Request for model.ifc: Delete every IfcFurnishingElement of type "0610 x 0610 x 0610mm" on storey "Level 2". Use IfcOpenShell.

First a look at what the model holds.

```python
import ifcopenshell
import ifcopenshell.util.element

model = ifcopenshell.open("model.ifc")
print(model.schema)
storey = next(s for s in model.by_type("IfcBuildingStorey") if s.Name == "Level 2")
furniture = [e for e in ifcopenshell.util.element.get_decomposition(storey) if e.is_a("IfcFurnishingElement")]
seen = {}
for e in furniture:
    element_type = ifcopenshell.util.element.get_type(e)
    name = element_type.Name if element_type not in (None, e) else None
    seen[name] = seen.get(name, 0) + 1
for name, count in sorted(seen.items(), key=str):
    print(count, "x", name)
```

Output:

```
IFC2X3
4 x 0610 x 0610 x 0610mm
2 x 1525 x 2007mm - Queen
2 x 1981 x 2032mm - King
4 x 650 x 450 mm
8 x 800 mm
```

```python
import ifcopenshell
import ifcopenshell.api.root
import ifcopenshell.util.element

model = ifcopenshell.open("model.ifc")

storey = next(s for s in model.by_type("IfcBuildingStorey") if s.Name == "Level 2")
furniture = [e for e in ifcopenshell.util.element.get_decomposition(storey) if e.is_a("IfcFurnishingElement")]
targets = [e for e in furniture if (t := ifcopenshell.util.element.get_type(e)) not in (None, e) and t.Name == "0610 x 0610 x 0610mm"]

for e in targets:
    ifcopenshell.api.root.remove_product(model, product=e)
print(len(targets), "removed")

model.write("model_rev.ifc")
```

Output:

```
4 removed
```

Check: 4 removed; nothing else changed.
